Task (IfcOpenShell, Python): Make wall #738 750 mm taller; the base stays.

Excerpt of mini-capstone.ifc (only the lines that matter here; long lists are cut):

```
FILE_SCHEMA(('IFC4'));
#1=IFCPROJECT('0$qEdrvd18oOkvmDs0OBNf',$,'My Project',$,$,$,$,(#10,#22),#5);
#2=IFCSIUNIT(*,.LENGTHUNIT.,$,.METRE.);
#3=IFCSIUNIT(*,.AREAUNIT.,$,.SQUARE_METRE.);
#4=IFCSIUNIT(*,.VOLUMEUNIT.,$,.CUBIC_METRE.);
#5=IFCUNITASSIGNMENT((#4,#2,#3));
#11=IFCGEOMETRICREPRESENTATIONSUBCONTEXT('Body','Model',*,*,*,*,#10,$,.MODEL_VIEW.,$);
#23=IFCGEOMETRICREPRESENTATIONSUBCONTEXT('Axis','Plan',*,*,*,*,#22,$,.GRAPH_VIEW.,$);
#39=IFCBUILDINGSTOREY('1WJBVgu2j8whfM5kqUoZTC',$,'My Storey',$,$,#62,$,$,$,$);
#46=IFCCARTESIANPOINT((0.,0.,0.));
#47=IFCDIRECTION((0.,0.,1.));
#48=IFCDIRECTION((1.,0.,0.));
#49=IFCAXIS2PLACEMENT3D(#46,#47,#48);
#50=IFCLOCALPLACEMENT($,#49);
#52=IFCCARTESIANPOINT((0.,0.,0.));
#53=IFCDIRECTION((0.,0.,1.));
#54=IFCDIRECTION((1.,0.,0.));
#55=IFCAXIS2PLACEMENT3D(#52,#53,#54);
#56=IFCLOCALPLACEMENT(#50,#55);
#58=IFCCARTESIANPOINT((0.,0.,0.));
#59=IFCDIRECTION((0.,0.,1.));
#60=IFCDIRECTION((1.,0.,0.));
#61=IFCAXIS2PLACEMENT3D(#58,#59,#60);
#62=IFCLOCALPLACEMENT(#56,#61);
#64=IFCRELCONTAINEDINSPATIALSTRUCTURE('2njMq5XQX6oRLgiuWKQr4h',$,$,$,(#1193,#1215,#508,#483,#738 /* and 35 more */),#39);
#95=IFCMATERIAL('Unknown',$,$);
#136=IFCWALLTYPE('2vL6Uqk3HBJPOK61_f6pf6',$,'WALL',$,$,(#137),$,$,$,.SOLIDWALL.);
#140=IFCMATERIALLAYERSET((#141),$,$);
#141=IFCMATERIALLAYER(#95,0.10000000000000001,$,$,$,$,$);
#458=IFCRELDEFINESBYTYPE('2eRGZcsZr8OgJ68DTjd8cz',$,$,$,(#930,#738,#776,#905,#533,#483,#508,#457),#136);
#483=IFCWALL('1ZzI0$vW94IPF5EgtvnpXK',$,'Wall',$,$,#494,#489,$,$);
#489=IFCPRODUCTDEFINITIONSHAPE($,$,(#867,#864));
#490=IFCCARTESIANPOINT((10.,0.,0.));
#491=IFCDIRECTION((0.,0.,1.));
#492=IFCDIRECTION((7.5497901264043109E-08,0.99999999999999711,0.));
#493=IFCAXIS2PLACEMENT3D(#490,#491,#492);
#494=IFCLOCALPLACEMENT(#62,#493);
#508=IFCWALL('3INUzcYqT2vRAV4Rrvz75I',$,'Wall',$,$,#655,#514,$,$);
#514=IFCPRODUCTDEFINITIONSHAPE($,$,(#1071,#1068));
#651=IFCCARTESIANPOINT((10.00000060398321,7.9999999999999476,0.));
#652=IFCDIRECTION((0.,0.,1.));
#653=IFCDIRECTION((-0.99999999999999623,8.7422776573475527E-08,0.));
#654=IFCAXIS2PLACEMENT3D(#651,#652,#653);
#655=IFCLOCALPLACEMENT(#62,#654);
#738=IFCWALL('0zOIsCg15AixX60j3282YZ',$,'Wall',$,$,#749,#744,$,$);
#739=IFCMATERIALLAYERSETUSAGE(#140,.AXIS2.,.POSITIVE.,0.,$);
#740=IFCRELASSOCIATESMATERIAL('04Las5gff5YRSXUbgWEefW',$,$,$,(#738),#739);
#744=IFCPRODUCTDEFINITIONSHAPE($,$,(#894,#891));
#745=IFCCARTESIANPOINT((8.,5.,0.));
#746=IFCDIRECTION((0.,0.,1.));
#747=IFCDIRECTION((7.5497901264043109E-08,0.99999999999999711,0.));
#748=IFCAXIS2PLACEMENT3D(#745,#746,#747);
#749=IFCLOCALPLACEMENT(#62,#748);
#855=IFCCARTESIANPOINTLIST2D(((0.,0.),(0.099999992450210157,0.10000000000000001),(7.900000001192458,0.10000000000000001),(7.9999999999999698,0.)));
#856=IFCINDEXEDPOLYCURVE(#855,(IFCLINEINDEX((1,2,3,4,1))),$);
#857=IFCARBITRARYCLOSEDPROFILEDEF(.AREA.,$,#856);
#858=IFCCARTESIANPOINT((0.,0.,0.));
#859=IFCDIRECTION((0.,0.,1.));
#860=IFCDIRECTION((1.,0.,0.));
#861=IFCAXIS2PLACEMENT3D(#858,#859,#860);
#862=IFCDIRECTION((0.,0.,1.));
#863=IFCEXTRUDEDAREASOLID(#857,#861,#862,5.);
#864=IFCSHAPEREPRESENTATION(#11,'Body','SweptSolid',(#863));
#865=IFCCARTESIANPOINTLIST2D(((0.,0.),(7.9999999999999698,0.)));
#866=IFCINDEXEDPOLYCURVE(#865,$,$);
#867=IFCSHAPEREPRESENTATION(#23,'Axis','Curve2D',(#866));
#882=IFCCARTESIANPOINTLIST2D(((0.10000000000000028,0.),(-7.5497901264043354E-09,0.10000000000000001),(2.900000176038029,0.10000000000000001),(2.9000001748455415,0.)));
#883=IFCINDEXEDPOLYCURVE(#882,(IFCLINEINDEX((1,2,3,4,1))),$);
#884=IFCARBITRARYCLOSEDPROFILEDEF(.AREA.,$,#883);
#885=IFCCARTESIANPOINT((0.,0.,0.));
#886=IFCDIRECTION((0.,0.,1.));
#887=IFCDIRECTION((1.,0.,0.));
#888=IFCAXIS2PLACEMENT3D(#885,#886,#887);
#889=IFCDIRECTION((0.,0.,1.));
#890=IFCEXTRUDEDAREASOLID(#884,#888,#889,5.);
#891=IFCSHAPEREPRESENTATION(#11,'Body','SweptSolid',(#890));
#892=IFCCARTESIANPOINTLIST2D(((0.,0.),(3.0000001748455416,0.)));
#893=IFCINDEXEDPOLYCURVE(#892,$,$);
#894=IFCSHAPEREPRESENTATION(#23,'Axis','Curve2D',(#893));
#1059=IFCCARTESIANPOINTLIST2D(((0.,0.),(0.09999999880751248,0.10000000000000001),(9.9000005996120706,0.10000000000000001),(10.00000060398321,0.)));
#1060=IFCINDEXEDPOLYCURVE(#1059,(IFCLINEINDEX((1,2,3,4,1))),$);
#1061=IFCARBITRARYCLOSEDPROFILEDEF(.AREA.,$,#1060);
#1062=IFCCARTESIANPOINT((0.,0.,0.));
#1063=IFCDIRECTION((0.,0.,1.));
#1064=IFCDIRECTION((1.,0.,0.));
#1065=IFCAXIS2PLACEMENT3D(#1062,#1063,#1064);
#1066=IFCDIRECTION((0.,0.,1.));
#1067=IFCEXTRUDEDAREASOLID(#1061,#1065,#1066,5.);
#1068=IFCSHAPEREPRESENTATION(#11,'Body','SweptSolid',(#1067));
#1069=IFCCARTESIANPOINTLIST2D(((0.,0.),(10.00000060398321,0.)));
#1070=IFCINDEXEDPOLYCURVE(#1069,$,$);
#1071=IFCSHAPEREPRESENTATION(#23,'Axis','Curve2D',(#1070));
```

```python
import ifcopenshell
import ifcopenshell.geom
import ifcopenshell.util.representation
import ifcopenshell.util.shape

model = ifcopenshell.open("mini-capstone.ifc")
settings = ifcopenshell.geom.settings()


def volume(element):
    """Net volume in cubic metres, openings subtracted."""
    shape = ifcopenshell.geom.create_shape(settings, element)
    return ifcopenshell.util.shape.get_volume(shape.geometry)


wall = model.by_guid("0zOIsCg15AixX60j3282YZ")
before = volume(wall)

body = ifcopenshell.util.representation.get_representation(wall, "Model", "Body")
solid = body.Items[0]
old_height = solid.Depth
solid.Depth += 0.75
after = volume(wall)

print(f"height {old_height:g} -> {solid.Depth:g}, volume {before:.3f} -> {after:.3f} m3")

model.write("mini-capstone-out.ifc")
```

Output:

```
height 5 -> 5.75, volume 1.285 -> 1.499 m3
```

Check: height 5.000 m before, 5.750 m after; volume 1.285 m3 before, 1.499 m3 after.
